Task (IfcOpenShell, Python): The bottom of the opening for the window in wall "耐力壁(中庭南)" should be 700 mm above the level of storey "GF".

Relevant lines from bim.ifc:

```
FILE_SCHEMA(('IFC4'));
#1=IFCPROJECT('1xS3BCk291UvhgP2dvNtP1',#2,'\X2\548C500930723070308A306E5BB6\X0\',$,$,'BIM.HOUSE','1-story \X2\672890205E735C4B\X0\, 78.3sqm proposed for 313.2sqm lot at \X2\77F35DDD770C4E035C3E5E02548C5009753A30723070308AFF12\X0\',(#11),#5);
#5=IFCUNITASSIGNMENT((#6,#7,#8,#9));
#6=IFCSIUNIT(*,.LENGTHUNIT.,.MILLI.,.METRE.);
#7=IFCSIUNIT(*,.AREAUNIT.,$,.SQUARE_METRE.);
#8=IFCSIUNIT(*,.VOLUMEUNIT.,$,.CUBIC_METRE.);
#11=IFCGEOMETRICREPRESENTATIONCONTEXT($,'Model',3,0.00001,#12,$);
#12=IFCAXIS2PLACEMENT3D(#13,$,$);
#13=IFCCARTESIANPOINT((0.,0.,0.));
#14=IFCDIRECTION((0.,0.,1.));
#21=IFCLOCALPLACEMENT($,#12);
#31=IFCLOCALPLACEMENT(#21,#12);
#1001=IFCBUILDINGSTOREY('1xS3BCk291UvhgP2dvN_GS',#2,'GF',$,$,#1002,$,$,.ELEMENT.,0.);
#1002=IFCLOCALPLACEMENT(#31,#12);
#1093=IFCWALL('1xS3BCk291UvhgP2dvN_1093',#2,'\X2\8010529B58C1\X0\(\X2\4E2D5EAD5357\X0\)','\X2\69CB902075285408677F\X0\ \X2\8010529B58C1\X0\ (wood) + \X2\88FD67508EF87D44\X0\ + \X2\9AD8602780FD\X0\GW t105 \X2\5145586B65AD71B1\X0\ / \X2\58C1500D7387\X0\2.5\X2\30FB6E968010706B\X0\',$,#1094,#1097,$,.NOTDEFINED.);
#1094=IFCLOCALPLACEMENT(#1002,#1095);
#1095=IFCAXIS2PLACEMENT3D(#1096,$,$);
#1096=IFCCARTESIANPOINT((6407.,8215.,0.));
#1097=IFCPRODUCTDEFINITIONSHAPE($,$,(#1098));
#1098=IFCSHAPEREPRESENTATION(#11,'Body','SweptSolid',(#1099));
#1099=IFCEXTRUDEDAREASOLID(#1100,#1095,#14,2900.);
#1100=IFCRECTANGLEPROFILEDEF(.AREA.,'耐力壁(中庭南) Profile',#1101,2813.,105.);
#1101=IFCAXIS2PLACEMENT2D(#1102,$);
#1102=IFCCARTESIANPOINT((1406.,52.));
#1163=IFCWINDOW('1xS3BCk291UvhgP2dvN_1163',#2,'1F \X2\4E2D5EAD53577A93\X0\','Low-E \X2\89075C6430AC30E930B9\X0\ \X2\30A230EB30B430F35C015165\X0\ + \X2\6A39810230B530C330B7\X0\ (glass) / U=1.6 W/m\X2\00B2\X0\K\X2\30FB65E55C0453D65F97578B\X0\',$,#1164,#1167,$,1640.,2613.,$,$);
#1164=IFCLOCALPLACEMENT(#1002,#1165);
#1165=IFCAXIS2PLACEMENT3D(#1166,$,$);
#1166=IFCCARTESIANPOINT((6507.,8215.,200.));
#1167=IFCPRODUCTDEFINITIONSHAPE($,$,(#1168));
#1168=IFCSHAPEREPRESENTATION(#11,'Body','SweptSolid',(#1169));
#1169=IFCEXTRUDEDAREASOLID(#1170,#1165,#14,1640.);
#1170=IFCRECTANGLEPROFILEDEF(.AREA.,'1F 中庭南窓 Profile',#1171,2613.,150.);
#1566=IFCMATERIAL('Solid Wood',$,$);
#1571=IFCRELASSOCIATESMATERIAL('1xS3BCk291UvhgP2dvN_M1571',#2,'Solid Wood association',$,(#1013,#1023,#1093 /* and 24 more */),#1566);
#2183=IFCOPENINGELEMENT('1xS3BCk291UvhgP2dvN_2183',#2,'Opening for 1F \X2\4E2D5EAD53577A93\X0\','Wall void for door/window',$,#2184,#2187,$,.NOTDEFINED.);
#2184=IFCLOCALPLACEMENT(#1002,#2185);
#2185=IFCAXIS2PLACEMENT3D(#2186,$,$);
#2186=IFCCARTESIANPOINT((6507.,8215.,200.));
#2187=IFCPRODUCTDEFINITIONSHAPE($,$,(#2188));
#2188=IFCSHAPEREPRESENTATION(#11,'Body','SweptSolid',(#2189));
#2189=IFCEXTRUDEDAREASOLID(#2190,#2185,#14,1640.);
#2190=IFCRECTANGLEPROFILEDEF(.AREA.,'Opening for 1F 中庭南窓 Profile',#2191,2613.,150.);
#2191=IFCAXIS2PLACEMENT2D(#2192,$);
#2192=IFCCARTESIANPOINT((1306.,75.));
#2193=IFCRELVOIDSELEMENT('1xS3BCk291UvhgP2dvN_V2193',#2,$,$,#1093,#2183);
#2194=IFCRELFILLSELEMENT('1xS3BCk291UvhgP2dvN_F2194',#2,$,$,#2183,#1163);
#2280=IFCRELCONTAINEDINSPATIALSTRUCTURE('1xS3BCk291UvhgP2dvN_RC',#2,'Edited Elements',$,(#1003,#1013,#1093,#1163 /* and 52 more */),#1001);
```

```python
import numpy as np
import ifcopenshell
import ifcopenshell.api.geometry
import ifcopenshell.geom
import ifcopenshell.util.element
import ifcopenshell.util.placement
import ifcopenshell.util.shape
import ifcopenshell.util.unit

model = ifcopenshell.open("bim.ifc")
unit_scale = ifcopenshell.util.unit.calculate_unit_scale(model)

window = model.by_id(1163)
opening = window.FillsVoids[0].RelatingOpeningElement
storey = ifcopenshell.util.element.get_container(window, ifc_class="IfcBuildingStorey")
level = ifcopenshell.util.placement.get_local_placement(storey.ObjectPlacement)[2, 3]

# The opening's origin need not be at the sill, so measure its lowest point.
shape = ifcopenshell.geom.create_shape(ifcopenshell.geom.settings(), opening)
bottom = ifcopenshell.util.shape.get_shape_bottom_elevation(shape, shape.geometry) / unit_scale
dz = level + 0.7 / unit_scale - bottom

shift = np.array([0.0, 0.0, dz])
# The window is not placed relative to its opening, so move both.
for product in (opening, window):
    matrix = ifcopenshell.util.placement.get_local_placement(product.ObjectPlacement)
    matrix[:3, 3] += shift
    ifcopenshell.api.geometry.edit_object_placement(model, product=product, matrix=matrix, is_si=False)

print(f"moved by {dz * unit_scale:+.3f} m")

model.write("bim-out.ifc")
```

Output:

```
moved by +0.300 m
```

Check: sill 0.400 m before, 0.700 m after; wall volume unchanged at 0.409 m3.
